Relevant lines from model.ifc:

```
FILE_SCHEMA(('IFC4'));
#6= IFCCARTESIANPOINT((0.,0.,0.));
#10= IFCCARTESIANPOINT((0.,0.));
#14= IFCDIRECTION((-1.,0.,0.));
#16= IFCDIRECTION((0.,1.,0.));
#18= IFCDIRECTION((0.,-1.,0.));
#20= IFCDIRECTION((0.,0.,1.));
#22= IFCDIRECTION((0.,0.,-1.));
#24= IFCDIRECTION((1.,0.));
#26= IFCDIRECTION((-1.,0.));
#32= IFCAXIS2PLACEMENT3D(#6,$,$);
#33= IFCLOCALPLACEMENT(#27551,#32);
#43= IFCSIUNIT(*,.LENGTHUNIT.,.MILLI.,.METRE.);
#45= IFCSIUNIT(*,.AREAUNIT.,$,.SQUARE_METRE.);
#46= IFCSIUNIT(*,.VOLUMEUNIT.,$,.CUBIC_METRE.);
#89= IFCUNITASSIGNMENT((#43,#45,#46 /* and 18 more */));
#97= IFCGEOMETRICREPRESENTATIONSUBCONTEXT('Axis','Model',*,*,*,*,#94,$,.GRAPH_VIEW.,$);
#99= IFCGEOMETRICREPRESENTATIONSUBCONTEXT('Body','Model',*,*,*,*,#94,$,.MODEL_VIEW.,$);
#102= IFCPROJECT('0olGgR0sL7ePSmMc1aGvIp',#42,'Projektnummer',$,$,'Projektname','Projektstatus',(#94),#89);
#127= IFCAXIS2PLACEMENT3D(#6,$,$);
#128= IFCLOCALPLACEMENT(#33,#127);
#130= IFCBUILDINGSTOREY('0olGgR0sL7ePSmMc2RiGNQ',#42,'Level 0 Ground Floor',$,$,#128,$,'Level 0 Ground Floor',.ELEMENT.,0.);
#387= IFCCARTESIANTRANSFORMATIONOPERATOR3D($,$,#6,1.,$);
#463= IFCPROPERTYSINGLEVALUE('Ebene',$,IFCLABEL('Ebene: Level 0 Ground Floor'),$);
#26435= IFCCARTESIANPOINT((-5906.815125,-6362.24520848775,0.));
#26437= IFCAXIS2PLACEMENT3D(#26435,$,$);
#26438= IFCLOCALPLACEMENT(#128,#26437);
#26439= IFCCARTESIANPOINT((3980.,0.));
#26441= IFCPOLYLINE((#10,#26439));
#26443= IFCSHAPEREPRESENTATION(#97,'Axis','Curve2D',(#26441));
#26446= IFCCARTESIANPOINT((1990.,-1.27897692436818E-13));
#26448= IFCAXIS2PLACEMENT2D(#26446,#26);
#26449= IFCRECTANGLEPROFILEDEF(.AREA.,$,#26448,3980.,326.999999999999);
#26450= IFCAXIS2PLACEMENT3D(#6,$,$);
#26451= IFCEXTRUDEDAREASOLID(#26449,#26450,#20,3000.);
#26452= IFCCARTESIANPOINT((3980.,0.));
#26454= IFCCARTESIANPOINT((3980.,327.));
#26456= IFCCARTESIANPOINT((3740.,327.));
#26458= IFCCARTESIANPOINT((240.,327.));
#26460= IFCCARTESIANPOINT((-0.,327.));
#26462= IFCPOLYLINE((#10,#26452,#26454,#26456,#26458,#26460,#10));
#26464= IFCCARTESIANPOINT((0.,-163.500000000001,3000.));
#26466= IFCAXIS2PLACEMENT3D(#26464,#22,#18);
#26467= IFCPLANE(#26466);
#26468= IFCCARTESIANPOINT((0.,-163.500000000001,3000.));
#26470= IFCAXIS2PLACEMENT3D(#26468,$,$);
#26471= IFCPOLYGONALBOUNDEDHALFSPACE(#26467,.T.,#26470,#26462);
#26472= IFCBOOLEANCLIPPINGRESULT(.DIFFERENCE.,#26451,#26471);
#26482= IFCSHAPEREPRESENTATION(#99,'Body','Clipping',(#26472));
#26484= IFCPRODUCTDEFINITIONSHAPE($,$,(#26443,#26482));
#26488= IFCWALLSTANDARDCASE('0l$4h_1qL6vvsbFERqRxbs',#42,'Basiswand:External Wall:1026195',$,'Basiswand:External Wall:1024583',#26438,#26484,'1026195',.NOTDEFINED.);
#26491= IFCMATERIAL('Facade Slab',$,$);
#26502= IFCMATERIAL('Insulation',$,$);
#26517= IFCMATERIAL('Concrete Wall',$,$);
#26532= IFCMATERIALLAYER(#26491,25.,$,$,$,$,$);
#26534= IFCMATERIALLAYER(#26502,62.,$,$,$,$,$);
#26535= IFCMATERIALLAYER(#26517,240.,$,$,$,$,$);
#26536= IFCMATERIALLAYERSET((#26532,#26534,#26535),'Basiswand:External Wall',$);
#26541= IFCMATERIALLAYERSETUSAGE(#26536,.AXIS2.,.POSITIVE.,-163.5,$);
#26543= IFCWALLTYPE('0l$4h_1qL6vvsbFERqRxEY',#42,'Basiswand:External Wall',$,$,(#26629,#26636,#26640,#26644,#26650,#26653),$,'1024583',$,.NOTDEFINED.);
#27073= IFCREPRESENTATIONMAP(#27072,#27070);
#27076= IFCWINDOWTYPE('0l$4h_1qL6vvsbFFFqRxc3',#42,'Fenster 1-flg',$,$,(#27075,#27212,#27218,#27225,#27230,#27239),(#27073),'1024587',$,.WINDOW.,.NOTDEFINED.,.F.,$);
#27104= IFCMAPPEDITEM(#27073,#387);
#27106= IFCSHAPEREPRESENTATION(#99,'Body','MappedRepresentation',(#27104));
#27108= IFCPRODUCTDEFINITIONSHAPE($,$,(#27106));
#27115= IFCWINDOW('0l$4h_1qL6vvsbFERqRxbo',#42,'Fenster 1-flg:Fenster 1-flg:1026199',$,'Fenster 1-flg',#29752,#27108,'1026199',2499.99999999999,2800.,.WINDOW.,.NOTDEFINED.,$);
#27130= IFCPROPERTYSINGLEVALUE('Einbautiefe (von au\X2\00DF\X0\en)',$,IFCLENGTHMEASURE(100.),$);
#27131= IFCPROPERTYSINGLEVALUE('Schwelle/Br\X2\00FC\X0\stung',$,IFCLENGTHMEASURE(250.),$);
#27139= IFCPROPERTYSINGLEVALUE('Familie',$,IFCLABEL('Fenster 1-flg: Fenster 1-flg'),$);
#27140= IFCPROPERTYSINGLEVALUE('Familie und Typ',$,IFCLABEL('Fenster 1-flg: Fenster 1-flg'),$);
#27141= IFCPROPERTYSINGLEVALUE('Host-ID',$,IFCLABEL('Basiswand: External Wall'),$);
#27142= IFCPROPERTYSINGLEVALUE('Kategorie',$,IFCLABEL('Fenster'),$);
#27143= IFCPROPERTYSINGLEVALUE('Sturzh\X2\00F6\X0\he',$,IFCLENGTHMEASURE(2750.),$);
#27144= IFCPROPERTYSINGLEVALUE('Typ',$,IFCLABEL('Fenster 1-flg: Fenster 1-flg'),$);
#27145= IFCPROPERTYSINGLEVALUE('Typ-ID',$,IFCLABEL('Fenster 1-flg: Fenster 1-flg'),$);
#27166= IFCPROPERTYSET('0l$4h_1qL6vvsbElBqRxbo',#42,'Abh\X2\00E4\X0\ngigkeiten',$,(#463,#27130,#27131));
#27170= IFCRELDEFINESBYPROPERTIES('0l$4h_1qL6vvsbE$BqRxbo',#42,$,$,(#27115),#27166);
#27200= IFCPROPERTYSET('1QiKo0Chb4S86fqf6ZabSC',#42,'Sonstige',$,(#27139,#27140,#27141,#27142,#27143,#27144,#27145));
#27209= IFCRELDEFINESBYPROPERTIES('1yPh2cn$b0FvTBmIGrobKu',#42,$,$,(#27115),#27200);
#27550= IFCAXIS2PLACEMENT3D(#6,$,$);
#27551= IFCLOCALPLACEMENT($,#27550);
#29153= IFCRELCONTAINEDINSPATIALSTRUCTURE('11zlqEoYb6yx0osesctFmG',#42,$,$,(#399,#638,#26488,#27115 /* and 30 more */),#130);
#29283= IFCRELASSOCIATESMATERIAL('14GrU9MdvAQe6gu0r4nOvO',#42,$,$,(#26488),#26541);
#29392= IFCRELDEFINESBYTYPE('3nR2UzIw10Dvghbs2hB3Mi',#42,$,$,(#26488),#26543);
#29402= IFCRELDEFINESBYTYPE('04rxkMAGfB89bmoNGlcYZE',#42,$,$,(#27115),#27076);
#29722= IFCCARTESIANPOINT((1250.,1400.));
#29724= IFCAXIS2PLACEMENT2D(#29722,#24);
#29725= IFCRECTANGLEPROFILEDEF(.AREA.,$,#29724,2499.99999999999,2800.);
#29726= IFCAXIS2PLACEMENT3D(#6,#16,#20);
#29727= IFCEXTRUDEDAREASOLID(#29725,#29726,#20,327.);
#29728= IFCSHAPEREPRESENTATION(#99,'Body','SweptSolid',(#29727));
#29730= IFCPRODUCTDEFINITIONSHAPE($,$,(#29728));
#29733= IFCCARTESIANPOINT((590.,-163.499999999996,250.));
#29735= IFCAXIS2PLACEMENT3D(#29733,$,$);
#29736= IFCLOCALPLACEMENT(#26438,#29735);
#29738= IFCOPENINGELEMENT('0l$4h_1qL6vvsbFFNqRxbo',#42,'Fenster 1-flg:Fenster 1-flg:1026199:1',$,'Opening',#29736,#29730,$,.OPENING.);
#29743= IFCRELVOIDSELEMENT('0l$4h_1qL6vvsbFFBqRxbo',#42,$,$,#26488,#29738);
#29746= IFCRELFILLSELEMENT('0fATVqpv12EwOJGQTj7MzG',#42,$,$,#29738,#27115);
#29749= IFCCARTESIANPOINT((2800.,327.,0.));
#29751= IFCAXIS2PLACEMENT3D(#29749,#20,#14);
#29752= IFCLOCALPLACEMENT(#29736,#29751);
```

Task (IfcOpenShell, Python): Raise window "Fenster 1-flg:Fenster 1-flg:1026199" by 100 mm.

```python
import numpy as np
import ifcopenshell
import ifcopenshell.api.geometry
import ifcopenshell.api.pset
import ifcopenshell.util.element
import ifcopenshell.util.placement
import ifcopenshell.util.unit

model = ifcopenshell.open("model.ifc")
unit_scale = ifcopenshell.util.unit.calculate_unit_scale(model)

window = model.by_guid("0l$4h_1qL6vvsbFERqRxbo")
opening = window.FillsVoids[0].RelatingOpeningElement
dz = 0.1 / unit_scale

shift = np.array([0.0, 0.0, dz])
# The window is placed relative to its opening, so it follows when the opening moves.
matrix = ifcopenshell.util.placement.get_local_placement(opening.ObjectPlacement)
matrix[:3, 3] += shift
ifcopenshell.api.geometry.edit_object_placement(
    model, product=opening, matrix=matrix, is_si=False, should_transform_children=True
)

# Keep the stored heights in step.
pset = model.by_id(ifcopenshell.util.element.get_pset(window, "Abhängigkeiten", should_inherit=False)["id"])
ifcopenshell.api.pset.edit_pset(model, pset=pset, properties={
    "Schwelle/Brüstung": model.create_entity("IfcLengthMeasure", ifcopenshell.util.element.get_pset(window, "Abhängigkeiten", "Schwelle/Brüstung") + dz),
})
pset = model.by_id(ifcopenshell.util.element.get_pset(window, "Sonstige", should_inherit=False)["id"])
ifcopenshell.api.pset.edit_pset(model, pset=pset, properties={
    "Sturzhöhe": model.create_entity("IfcLengthMeasure", ifcopenshell.util.element.get_pset(window, "Sonstige", "Sturzhöhe") + dz),
})

print(f"moved by {dz * unit_scale:+.3f} m")

model.write("model-out.ifc")
```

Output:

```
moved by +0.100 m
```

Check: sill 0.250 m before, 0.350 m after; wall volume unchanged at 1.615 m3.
